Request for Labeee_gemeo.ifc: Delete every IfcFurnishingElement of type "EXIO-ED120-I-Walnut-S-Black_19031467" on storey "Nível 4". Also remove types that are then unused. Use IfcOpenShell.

First a look at what the model holds.

```python
import ifcopenshell
import ifcopenshell.util.element

model = ifcopenshell.open("Labeee_gemeo.ifc")
print(model.schema)
storey = next(s for s in model.by_type("IfcBuildingStorey") if s.Name == "Nível 4")
furniture = [e for e in ifcopenshell.util.element.get_decomposition(storey) if e.is_a("IfcFurnishingElement")]
seen = {}
for e in furniture:
    element_type = ifcopenshell.util.element.get_type(e)
    name = element_type.Name if element_type not in (None, e) else None
    seen[name] = seen.get(name, 0) + 1
for name, count in sorted(seen.items(), key=str):
    print(count, "x", name)
```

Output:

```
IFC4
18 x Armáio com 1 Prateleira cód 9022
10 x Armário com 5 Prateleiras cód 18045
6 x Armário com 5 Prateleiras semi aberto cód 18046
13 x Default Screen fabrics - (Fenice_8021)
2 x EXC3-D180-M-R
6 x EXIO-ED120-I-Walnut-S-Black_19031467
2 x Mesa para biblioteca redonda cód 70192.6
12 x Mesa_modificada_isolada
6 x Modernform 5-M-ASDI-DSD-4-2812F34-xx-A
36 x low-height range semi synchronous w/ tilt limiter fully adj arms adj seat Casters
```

```python
import ifcopenshell
import ifcopenshell.api.root
import ifcopenshell.util.element

model = ifcopenshell.open("Labeee_gemeo.ifc")

storey = next(s for s in model.by_type("IfcBuildingStorey") if s.Name == "Nível 4")
furniture = [e for e in ifcopenshell.util.element.get_decomposition(storey) if e.is_a("IfcFurnishingElement")]
targets = [e for e in furniture if (t := ifcopenshell.util.element.get_type(e)) not in (None, e) and t.Name == "EXIO-ED120-I-Walnut-S-Black_19031467"]
types = {ifcopenshell.util.element.get_type(e) for e in targets} - {None, *targets}

for e in targets:
    ifcopenshell.api.root.remove_product(model, product=e)
print(len(targets), "removed")

unused = [t for t in types if not ifcopenshell.util.element.get_types(t)]
for t in unused:
    ifcopenshell.api.root.remove_product(model, product=t)
print(len(unused), "unused types removed")

model.write("Labeee_gemeo_updated.ifc")
```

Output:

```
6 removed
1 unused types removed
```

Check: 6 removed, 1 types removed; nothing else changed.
